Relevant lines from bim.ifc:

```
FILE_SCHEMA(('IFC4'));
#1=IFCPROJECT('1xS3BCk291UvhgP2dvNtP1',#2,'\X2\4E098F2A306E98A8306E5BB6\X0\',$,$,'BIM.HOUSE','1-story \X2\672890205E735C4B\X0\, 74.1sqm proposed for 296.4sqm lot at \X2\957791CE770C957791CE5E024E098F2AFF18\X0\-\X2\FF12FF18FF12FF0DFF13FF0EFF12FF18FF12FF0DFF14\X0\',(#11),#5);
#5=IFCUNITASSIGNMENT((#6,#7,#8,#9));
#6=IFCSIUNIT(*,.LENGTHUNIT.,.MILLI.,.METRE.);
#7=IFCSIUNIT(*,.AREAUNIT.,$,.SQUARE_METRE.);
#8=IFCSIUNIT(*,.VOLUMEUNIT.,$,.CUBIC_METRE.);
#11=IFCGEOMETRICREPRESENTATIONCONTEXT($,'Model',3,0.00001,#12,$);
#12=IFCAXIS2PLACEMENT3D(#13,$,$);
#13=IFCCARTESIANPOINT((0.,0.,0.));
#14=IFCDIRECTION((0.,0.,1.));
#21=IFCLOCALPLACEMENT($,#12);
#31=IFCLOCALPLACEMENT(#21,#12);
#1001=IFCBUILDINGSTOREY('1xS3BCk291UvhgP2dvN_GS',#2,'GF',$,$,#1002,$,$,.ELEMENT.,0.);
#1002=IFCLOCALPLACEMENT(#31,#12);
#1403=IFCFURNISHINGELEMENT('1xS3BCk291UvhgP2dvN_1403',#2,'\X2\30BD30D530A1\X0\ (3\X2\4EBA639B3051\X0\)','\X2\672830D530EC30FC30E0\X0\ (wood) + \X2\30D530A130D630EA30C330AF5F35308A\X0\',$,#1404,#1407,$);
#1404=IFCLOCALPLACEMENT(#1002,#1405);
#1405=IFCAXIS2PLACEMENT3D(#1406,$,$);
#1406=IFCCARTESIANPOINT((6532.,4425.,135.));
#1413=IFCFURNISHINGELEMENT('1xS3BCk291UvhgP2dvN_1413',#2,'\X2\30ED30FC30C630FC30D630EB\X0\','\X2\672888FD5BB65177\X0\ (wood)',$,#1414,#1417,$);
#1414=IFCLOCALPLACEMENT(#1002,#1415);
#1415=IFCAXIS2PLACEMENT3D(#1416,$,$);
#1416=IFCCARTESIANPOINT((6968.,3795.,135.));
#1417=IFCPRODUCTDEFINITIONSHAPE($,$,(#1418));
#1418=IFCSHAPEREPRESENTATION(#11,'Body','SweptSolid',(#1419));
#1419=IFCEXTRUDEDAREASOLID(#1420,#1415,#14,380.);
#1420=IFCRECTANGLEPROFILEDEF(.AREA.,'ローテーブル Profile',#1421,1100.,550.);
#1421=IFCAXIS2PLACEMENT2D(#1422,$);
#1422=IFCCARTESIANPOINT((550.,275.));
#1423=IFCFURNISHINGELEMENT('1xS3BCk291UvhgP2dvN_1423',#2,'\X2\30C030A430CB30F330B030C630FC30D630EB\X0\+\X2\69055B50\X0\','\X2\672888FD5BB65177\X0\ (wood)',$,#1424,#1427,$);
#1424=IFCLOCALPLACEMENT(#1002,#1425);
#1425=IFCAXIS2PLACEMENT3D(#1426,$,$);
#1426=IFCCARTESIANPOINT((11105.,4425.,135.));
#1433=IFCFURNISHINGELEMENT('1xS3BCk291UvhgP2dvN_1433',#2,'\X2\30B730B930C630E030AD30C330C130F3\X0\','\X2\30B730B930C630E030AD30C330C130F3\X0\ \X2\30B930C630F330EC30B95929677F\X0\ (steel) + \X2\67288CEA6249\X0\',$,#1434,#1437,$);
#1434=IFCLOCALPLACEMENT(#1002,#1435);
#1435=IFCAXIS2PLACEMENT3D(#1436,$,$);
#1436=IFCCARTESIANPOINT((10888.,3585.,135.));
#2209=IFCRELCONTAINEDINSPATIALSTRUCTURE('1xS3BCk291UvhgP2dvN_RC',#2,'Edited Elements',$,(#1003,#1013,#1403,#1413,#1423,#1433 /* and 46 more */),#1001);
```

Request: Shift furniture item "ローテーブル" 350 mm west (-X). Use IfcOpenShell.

```python
import ifcopenshell
import ifcopenshell.api.geometry
import ifcopenshell.util.placement

model = ifcopenshell.open("bim.ifc")

item = model.by_guid("1xS3BCk291UvhgP2dvN_1413")
matrix = ifcopenshell.util.placement.get_local_placement(item.ObjectPlacement)
matrix[0, 3] -= 350.0
ifcopenshell.api.geometry.edit_object_placement(model, product=item, matrix=matrix, is_si=False)

print(ifcopenshell.util.placement.get_local_placement(item.ObjectPlacement).round(3) + 0.0)

model.write("bim_v2.ifc")
```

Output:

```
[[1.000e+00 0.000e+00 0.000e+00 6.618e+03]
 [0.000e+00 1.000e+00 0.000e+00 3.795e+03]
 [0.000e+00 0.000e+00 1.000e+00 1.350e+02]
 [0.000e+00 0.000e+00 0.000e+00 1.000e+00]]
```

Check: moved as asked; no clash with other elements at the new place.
